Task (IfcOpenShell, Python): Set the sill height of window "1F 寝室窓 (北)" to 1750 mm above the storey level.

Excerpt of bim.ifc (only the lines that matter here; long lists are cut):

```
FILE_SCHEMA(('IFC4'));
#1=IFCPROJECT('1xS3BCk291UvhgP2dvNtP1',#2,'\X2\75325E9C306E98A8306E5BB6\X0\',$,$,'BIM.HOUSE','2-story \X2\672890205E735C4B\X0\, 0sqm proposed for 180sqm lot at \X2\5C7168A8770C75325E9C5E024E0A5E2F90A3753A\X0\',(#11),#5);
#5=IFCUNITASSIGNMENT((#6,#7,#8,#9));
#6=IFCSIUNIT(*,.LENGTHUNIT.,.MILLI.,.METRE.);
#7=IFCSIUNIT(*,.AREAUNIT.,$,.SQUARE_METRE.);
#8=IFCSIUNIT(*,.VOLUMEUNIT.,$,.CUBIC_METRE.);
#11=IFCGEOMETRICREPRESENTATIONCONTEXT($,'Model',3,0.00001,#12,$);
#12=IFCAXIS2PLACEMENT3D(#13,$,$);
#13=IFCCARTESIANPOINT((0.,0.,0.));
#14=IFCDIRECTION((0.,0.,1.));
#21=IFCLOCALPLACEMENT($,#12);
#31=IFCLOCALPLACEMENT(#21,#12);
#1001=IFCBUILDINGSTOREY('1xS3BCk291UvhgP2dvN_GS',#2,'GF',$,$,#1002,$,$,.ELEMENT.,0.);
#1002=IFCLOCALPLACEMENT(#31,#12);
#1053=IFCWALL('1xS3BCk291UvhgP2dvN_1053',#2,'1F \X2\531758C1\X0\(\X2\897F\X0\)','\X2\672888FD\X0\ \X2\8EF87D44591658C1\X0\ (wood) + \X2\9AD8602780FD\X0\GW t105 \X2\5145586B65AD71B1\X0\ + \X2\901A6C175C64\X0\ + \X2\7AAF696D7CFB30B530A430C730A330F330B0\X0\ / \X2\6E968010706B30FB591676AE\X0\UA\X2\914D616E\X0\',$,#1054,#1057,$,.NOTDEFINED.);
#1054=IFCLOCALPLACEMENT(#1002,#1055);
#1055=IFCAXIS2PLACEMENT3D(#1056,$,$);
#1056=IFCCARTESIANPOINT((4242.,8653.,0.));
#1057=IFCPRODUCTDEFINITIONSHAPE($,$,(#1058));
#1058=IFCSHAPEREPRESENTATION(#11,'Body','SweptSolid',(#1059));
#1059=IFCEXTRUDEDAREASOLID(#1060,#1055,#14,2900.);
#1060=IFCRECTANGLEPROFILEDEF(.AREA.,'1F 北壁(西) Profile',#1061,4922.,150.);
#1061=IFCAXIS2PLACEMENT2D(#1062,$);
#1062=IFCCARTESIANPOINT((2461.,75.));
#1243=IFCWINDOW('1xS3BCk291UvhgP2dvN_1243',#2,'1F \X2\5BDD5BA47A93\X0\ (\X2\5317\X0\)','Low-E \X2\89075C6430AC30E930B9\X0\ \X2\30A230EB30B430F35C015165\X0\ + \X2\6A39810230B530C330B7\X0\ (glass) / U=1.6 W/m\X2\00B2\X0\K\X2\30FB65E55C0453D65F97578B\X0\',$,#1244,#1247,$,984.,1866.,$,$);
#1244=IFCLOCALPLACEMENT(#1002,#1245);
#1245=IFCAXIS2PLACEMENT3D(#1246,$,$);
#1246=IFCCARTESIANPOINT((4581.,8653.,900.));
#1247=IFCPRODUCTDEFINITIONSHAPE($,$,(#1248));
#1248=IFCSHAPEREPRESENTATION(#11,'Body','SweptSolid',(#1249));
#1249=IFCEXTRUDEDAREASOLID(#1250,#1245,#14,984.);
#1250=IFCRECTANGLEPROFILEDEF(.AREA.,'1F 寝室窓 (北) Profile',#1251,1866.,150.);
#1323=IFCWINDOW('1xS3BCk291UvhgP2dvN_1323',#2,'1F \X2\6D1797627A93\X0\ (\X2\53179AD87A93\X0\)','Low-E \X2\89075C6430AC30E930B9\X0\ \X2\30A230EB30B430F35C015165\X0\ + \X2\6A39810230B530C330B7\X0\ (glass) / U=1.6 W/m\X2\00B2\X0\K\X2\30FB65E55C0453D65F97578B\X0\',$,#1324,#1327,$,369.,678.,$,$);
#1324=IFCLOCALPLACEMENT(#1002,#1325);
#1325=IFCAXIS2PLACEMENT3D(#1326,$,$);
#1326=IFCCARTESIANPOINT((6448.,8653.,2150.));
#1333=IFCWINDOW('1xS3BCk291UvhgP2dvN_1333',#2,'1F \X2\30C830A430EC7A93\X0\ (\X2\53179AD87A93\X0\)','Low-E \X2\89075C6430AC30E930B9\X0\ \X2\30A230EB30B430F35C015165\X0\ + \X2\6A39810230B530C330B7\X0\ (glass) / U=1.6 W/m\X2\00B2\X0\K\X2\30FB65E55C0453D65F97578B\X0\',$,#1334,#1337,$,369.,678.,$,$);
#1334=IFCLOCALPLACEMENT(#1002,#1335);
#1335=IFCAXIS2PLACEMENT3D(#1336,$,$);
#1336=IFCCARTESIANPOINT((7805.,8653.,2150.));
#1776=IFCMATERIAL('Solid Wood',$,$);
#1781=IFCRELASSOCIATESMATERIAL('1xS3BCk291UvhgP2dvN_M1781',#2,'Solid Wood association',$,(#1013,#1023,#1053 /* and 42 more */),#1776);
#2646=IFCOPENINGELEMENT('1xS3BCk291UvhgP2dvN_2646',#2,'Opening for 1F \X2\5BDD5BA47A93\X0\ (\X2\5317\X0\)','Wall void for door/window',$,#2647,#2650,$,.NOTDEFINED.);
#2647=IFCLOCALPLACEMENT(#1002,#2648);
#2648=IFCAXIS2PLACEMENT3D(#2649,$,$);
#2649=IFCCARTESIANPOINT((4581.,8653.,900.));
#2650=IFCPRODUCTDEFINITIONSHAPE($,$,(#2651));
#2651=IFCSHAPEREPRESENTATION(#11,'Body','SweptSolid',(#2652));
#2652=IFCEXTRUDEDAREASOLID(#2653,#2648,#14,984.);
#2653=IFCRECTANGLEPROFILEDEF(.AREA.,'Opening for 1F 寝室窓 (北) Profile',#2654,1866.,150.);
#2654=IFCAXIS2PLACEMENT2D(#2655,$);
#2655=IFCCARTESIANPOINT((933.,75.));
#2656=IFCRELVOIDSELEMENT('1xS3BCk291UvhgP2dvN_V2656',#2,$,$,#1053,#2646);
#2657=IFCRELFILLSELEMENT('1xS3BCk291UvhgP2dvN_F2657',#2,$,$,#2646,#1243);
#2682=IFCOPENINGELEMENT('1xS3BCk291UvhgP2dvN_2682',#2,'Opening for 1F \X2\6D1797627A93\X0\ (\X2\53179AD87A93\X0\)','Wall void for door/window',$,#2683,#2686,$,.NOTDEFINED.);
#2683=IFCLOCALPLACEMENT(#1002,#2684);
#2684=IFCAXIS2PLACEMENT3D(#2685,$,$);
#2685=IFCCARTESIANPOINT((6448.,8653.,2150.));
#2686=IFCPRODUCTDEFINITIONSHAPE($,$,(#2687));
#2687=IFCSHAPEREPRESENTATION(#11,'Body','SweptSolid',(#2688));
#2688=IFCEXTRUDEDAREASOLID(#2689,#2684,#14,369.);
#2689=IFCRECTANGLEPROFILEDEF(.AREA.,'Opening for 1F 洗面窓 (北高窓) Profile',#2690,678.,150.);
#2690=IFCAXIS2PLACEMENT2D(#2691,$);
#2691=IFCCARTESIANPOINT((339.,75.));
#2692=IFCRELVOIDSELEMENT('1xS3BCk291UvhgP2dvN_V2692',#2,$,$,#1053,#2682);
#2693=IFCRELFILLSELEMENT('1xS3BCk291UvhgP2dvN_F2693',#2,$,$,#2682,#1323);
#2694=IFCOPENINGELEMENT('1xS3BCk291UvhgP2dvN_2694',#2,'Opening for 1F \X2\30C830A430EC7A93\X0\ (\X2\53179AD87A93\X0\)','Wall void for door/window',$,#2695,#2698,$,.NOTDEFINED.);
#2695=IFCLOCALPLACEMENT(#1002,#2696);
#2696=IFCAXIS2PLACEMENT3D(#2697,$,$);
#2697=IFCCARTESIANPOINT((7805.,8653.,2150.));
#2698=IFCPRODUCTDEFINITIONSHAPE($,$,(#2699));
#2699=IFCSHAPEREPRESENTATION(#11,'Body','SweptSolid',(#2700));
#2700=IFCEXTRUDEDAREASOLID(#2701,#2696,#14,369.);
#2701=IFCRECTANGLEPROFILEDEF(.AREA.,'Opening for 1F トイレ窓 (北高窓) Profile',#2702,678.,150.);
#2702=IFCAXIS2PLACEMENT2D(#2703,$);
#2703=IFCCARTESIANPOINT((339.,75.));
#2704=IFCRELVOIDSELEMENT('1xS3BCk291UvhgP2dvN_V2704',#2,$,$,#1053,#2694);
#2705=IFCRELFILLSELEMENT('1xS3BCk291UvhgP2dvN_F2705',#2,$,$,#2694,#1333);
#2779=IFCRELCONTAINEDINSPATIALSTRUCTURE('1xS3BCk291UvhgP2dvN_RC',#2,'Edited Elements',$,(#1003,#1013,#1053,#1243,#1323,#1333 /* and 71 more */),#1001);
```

```python
import numpy as np
import ifcopenshell
import ifcopenshell.api.geometry
import ifcopenshell.geom
import ifcopenshell.util.element
import ifcopenshell.util.placement
import ifcopenshell.util.shape
import ifcopenshell.util.unit

model = ifcopenshell.open("bim.ifc")
unit_scale = ifcopenshell.util.unit.calculate_unit_scale(model)

window = model.by_guid("1xS3BCk291UvhgP2dvN_1243")
opening = window.FillsVoids[0].RelatingOpeningElement
storey = ifcopenshell.util.element.get_container(window, ifc_class="IfcBuildingStorey")
level = ifcopenshell.util.placement.get_local_placement(storey.ObjectPlacement)[2, 3]

# The opening's origin need not be at the sill, so measure its lowest point.
shape = ifcopenshell.geom.create_shape(ifcopenshell.geom.settings(), opening)
bottom = ifcopenshell.util.shape.get_shape_bottom_elevation(shape, shape.geometry) / unit_scale
dz = level + 1750.0 - bottom

shift = np.array([0.0, 0.0, dz])
# The window is not placed relative to its opening, so move both.
for product in (opening, window):
    matrix = ifcopenshell.util.placement.get_local_placement(product.ObjectPlacement)
    matrix[:3, 3] += shift
    ifcopenshell.api.geometry.edit_object_placement(model, product=product, matrix=matrix, is_si=False)

print(f"moved by {dz * unit_scale:+.3f} m")

model.write("bim_rev.ifc")
```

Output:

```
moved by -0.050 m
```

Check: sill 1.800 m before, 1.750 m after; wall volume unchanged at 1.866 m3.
